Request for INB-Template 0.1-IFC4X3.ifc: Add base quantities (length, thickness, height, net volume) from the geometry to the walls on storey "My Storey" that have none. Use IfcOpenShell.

First a look at what the model holds.

```python
import ifcopenshell
import ifcopenshell.util.element
import ifcopenshell.util.unit

model = ifcopenshell.open("INB-Template 0.1-IFC4X3.ifc")
print(model.schema)
for unit_type in ("LENGTHUNIT", "AREAUNIT", "VOLUMEUNIT"):
    print(unit_type, ifcopenshell.util.unit.calculate_unit_scale(model, unit_type))
storey = next(s for s in model.by_type("IfcBuildingStorey") if s.Name == "My Storey")
walls = [e for e in ifcopenshell.util.element.get_decomposition(storey) if e.is_a("IfcWall")]
for e in sorted(walls, key=lambda e: e.id()):
    print(e.id(), e.is_a(), e.Name, list(ifcopenshell.util.element.get_psets(e, qtos_only=True)), sep=" | ")
```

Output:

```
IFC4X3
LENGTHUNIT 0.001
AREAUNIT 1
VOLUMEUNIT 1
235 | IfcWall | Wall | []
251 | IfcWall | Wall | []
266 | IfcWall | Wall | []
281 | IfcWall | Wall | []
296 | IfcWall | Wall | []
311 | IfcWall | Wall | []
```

```python
import ifcopenshell
import ifcopenshell.api.pset
import ifcopenshell.geom
import ifcopenshell.util.element
import ifcopenshell.util.shape
import ifcopenshell.util.unit

model = ifcopenshell.open("INB-Template 0.1-IFC4X3.ifc")
unit_scale = ifcopenshell.util.unit.calculate_unit_scale(model)
volume_scale = ifcopenshell.util.unit.calculate_unit_scale(model, "VOLUMEUNIT")
settings = ifcopenshell.geom.settings()

storey = next(s for s in model.by_type("IfcBuildingStorey") if s.Name == "My Storey")
walls = [e for e in ifcopenshell.util.element.get_decomposition(storey) if e.is_a("IfcWall")]

for e in sorted(walls, key=lambda e: e.id()):
    if ifcopenshell.util.element.get_psets(e, qtos_only=True, should_inherit=False):
        continue
    # Geometry comes back in metres, in the element's own axes.
    shape = ifcopenshell.geom.create_shape(settings, e)
    values = {
        "Length": ifcopenshell.util.shape.get_x(shape.geometry) / unit_scale,
        "Width": ifcopenshell.util.shape.get_y(shape.geometry) / unit_scale,
        "Height": ifcopenshell.util.shape.get_z(shape.geometry) / unit_scale,
        "NetVolume": ifcopenshell.util.shape.get_volume(shape.geometry) / volume_scale,
    }
    qto = ifcopenshell.api.pset.add_qto(model, product=e, name="Qto_WallBaseQuantities")
    ifcopenshell.api.pset.edit_qto(model, qto=qto, properties=values)
    print(e.id(), {k: round(v, 3) for k, v in values.items()})

model.write("INB-Template 0.1-IFC4X3_edited.ifc")
```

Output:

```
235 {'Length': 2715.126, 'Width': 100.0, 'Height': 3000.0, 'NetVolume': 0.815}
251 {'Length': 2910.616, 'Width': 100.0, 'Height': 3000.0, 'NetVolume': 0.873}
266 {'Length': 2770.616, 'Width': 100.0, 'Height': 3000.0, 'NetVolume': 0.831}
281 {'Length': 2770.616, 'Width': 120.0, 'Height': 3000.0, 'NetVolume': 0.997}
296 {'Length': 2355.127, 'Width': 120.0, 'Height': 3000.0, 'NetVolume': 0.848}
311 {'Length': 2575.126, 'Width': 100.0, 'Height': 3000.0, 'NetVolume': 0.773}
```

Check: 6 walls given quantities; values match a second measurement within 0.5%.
